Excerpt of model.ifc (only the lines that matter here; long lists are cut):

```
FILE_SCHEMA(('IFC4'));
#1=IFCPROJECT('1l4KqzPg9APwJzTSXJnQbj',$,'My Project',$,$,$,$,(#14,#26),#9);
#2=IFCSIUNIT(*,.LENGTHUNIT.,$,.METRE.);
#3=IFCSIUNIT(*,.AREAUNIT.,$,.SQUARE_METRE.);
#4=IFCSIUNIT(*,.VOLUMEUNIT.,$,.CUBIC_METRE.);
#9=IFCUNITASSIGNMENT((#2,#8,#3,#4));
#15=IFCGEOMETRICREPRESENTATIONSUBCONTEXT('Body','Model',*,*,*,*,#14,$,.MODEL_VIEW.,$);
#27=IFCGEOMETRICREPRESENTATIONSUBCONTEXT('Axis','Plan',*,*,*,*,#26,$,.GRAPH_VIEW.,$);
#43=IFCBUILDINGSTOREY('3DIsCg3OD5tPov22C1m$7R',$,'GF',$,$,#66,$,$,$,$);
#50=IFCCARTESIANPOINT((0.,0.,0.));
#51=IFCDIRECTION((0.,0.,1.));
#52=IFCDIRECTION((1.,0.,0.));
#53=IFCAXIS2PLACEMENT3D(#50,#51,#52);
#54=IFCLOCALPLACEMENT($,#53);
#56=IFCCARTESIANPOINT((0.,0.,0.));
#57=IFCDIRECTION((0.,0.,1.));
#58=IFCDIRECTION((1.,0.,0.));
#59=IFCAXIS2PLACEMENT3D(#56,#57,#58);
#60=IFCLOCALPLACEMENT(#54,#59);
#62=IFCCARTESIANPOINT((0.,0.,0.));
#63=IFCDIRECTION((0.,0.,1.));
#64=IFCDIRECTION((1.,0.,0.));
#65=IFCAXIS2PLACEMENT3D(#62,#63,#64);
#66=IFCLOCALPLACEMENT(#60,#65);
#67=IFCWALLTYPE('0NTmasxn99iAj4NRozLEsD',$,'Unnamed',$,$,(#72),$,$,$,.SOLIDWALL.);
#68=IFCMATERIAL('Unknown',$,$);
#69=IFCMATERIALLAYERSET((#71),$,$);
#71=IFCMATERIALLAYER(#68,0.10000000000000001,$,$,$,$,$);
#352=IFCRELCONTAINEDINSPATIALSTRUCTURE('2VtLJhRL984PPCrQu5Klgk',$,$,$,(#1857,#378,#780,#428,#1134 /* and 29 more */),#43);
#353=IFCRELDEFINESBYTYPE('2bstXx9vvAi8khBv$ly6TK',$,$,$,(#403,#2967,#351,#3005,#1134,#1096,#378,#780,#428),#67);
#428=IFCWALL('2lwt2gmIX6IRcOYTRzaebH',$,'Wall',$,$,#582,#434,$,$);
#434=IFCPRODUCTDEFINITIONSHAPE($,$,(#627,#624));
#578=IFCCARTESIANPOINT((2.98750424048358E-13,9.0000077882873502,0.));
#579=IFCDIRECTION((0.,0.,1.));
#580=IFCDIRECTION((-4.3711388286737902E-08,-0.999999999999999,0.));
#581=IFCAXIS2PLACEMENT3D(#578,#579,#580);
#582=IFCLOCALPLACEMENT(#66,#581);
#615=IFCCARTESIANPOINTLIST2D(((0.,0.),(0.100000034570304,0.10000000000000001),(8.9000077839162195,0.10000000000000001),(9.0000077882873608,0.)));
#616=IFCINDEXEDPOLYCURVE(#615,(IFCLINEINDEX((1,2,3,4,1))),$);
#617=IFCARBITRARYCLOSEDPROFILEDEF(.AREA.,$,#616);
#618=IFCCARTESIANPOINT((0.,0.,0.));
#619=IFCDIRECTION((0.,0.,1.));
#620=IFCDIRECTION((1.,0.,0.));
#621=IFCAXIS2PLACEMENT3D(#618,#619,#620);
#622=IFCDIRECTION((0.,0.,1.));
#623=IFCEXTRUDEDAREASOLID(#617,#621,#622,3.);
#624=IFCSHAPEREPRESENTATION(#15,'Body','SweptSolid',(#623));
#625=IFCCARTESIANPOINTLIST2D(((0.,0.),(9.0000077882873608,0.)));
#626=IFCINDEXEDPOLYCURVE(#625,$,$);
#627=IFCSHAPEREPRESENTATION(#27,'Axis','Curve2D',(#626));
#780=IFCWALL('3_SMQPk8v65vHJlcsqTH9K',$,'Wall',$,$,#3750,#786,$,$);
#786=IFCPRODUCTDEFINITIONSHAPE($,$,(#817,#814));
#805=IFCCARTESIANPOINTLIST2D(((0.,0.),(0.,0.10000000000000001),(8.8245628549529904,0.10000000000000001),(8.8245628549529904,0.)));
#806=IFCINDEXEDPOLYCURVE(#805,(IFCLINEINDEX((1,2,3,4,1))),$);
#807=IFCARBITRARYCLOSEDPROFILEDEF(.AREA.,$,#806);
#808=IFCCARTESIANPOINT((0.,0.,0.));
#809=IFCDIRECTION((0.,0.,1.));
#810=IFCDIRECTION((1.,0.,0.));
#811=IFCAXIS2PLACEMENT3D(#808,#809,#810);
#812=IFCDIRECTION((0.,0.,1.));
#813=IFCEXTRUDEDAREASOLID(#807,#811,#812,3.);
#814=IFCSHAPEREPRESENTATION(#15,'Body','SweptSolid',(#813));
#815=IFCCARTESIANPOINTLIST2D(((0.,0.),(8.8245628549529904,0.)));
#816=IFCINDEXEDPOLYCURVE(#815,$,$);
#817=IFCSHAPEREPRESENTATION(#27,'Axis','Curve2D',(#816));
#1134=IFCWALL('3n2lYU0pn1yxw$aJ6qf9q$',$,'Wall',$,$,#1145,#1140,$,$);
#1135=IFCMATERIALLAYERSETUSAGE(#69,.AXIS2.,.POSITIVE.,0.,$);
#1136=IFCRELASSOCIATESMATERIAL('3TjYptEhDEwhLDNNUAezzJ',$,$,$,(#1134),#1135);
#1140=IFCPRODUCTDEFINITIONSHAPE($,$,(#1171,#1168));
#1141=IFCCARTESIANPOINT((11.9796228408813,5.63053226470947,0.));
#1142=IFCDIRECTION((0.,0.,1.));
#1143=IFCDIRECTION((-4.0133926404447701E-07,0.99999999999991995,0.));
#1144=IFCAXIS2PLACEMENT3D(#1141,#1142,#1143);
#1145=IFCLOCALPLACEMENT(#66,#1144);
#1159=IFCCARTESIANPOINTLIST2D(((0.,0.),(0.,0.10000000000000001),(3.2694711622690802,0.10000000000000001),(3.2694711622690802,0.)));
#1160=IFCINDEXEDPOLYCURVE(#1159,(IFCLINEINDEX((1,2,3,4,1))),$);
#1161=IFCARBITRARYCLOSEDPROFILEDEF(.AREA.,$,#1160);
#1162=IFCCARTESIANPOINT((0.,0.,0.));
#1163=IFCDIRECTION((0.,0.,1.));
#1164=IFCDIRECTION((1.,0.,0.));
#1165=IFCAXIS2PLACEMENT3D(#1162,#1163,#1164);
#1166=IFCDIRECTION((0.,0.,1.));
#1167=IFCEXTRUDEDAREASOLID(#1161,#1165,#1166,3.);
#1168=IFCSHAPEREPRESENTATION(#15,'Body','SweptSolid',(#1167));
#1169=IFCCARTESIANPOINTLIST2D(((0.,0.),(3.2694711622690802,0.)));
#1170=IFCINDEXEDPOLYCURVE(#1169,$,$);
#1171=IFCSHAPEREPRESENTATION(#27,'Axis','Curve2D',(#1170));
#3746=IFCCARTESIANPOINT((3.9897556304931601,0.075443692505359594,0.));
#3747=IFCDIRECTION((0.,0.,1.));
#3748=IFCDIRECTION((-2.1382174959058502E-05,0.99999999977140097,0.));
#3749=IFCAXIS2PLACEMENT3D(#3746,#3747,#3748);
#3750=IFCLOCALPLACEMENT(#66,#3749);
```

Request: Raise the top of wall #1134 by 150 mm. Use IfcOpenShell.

```python
import ifcopenshell
import ifcopenshell.geom
import ifcopenshell.util.representation
import ifcopenshell.util.shape
import ifcopenshell.util.unit

model = ifcopenshell.open("model.ifc")
unit_scale = ifcopenshell.util.unit.calculate_unit_scale(model)
settings = ifcopenshell.geom.settings()


def volume(element):
    """Net volume in cubic metres, openings subtracted."""
    shape = ifcopenshell.geom.create_shape(settings, element)
    return ifcopenshell.util.shape.get_volume(shape.geometry)


wall = model.by_guid("3n2lYU0pn1yxw$aJ6qf9q$")
before = volume(wall)

body = ifcopenshell.util.representation.get_representation(wall, "Model", "Body")
solid = body.Items[0]
old_height = solid.Depth
solid.Depth += 0.15 / unit_scale
after = volume(wall)

print(f"height {old_height:g} -> {solid.Depth:g}, volume {before:.3f} -> {after:.3f} m3")

model.write("model_rev.ifc")
```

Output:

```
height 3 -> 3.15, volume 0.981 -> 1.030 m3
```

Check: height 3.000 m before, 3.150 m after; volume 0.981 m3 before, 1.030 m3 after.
